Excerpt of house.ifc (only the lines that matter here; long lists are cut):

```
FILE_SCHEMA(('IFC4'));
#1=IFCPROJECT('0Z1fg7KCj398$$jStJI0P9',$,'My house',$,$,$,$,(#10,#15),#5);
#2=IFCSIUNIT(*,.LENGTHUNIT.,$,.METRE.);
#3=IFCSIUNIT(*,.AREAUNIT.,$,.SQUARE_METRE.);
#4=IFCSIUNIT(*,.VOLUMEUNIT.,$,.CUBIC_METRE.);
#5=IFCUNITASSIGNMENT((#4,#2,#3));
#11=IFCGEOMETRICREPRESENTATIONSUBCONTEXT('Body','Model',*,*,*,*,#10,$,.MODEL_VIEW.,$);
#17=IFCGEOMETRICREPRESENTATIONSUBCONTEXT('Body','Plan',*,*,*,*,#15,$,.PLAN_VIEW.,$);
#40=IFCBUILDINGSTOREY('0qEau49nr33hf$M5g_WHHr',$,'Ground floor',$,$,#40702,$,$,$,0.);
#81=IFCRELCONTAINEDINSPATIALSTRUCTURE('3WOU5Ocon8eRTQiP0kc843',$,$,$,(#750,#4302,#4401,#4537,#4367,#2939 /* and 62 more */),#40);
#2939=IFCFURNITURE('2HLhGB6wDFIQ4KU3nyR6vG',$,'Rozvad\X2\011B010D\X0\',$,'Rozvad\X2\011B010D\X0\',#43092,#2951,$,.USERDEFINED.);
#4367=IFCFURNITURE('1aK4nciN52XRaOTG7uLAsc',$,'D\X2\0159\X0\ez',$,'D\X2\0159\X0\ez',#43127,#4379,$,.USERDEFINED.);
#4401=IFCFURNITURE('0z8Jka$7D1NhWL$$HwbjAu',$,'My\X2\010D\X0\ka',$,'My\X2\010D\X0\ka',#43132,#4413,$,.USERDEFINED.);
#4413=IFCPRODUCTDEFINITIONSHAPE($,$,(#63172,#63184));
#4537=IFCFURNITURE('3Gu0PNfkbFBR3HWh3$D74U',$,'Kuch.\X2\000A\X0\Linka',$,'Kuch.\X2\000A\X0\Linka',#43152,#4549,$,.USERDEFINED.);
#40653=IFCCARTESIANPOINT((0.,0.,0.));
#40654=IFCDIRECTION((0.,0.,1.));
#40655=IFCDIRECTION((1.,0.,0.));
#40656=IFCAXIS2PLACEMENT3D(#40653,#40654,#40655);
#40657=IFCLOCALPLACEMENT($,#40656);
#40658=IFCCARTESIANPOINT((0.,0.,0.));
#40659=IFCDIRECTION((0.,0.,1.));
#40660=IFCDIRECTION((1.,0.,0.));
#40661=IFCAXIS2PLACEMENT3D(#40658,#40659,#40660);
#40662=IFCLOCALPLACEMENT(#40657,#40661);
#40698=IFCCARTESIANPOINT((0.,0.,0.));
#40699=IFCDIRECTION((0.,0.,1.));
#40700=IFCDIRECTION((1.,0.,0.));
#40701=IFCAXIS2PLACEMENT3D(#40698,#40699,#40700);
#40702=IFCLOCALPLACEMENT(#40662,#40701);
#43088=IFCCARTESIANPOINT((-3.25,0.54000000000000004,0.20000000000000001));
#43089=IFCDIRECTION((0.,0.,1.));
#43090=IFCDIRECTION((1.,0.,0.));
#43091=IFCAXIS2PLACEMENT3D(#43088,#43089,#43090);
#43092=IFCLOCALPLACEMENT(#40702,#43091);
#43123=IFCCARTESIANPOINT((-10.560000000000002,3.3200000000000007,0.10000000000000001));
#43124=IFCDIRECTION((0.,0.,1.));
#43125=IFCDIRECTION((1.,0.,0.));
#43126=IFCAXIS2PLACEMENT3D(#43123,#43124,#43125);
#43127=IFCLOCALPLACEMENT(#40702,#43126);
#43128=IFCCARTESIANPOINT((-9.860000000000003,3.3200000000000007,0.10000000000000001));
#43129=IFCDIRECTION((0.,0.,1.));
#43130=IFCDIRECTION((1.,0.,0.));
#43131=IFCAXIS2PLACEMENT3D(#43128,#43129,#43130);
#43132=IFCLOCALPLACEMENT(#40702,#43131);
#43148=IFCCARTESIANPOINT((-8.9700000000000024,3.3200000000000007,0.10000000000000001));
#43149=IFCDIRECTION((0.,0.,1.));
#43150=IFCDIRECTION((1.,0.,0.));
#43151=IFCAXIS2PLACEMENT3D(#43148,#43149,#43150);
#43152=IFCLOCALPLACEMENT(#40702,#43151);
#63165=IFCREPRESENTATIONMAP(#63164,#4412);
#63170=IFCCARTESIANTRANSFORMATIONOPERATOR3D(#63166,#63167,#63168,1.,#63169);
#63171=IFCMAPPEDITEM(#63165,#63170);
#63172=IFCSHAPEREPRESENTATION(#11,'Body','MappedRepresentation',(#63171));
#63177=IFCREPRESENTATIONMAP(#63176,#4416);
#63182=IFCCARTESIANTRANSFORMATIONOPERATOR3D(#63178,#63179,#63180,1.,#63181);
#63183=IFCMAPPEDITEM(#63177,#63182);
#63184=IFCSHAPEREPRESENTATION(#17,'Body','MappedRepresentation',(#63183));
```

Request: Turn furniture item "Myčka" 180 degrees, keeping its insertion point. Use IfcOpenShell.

```python
import ifcopenshell
import ifcopenshell.api.geometry
import ifcopenshell.util.placement

model = ifcopenshell.open("house.ifc")

item = model.by_guid("0z8Jka$7D1NhWL$$HwbjAu")
matrix = ifcopenshell.util.placement.get_local_placement(item.ObjectPlacement)
matrix = matrix @ ifcopenshell.util.placement.rotation(180, "Z")
ifcopenshell.api.geometry.edit_object_placement(model, product=item, matrix=matrix, is_si=False)

print(ifcopenshell.util.placement.get_local_placement(item.ObjectPlacement).round(3) + 0.0)

model.write("house_rev.ifc")
```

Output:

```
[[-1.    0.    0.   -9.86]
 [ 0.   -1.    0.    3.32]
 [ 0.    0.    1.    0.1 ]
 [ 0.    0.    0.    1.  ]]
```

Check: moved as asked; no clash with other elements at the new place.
